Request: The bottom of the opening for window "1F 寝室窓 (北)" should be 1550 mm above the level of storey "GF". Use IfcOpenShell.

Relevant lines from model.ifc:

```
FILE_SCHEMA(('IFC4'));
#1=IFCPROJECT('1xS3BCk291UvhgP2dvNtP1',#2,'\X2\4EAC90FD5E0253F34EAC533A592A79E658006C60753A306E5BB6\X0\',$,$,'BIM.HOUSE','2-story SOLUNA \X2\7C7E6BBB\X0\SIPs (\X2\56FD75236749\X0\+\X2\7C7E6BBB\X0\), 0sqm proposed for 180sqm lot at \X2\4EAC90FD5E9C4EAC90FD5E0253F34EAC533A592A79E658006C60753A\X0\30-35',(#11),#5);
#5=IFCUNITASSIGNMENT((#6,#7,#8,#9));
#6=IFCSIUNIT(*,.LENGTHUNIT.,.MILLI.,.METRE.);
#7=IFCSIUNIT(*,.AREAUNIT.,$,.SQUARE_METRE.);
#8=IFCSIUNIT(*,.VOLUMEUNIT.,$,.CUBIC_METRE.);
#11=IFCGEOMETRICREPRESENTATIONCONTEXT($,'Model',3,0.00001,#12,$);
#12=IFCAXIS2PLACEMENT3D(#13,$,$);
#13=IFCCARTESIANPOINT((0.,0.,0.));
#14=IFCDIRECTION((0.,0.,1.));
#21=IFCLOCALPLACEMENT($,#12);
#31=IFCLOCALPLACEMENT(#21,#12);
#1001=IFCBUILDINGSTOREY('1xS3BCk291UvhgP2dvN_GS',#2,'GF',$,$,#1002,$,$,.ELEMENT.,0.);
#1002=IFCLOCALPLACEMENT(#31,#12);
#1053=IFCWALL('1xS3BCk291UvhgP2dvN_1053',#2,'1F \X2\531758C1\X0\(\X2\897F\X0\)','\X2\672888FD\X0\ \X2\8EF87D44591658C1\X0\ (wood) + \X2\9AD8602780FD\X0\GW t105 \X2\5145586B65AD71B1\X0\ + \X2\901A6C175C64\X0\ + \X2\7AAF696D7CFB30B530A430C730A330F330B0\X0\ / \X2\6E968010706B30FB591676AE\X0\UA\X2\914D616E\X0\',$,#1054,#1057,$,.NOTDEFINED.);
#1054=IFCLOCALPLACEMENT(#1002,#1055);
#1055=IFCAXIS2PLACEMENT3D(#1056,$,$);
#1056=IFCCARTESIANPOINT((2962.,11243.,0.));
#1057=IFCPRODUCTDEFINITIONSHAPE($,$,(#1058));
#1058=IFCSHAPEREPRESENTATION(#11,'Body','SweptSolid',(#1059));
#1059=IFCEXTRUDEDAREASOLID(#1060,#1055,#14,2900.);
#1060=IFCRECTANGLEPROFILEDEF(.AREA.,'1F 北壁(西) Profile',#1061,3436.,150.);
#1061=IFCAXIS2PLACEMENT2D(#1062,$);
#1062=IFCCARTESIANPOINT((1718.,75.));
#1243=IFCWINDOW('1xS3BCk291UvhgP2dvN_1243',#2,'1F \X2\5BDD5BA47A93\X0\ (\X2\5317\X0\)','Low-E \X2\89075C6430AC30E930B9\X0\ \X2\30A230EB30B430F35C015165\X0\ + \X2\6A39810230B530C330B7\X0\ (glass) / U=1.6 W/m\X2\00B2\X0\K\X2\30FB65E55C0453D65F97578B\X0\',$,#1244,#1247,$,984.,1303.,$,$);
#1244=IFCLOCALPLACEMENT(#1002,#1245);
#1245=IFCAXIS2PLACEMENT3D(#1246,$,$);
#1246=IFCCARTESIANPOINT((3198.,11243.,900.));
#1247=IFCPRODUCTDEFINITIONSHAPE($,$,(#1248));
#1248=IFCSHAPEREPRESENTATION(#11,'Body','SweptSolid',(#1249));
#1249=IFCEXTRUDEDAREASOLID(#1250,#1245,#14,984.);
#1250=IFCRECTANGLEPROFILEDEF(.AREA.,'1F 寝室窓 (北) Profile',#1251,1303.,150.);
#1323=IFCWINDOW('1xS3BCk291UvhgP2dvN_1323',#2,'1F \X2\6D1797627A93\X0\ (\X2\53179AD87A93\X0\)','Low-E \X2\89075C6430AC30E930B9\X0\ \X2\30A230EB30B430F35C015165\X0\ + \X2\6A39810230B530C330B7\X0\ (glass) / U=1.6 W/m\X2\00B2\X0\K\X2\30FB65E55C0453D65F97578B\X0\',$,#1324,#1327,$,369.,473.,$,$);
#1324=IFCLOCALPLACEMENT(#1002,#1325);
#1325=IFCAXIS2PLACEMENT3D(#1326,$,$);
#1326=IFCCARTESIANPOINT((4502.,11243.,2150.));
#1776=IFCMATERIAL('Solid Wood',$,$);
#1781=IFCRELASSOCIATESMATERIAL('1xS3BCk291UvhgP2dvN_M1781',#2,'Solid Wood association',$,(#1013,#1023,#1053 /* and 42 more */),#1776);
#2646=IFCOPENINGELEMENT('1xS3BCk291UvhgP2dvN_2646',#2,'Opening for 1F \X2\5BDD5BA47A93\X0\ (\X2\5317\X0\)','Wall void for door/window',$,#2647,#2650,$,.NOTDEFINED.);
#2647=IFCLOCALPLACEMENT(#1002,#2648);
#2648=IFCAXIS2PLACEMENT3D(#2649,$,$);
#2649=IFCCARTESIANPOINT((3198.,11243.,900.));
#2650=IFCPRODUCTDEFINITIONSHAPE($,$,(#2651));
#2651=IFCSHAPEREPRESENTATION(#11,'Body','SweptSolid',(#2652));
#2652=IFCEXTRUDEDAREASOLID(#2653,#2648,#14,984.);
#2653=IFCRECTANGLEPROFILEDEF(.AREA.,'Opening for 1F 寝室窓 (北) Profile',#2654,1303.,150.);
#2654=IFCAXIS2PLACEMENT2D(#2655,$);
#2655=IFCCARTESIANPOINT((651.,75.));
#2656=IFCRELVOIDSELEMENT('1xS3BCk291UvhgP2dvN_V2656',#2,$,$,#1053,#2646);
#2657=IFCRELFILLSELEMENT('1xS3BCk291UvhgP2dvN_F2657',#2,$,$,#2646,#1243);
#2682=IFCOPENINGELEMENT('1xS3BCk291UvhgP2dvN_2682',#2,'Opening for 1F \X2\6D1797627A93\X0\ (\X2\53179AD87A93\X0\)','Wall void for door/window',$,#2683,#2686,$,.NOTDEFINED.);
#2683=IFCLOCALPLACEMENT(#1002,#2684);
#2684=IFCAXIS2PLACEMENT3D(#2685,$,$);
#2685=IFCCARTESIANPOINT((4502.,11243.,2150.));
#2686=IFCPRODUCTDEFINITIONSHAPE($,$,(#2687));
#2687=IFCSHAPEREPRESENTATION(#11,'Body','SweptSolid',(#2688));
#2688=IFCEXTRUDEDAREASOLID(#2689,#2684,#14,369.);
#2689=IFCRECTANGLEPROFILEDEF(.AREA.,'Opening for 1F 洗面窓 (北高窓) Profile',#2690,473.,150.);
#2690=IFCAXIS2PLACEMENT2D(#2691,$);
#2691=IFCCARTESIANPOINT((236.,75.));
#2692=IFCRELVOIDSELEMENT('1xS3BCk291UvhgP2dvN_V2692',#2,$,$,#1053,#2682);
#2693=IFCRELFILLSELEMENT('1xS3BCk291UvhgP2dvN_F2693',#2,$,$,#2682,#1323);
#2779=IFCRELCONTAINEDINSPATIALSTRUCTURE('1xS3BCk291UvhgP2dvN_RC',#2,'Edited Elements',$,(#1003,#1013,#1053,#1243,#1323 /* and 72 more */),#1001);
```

```python
import numpy as np
import ifcopenshell
import ifcopenshell.api.geometry
import ifcopenshell.geom
import ifcopenshell.util.element
import ifcopenshell.util.placement
import ifcopenshell.util.shape
import ifcopenshell.util.unit

model = ifcopenshell.open("model.ifc")
unit_scale = ifcopenshell.util.unit.calculate_unit_scale(model)

window = model.by_guid("1xS3BCk291UvhgP2dvN_1243")
opening = window.FillsVoids[0].RelatingOpeningElement
storey = ifcopenshell.util.element.get_container(window, ifc_class="IfcBuildingStorey")
level = ifcopenshell.util.placement.get_local_placement(storey.ObjectPlacement)[2, 3]

# The opening's origin need not be at the sill, so measure its lowest point.
shape = ifcopenshell.geom.create_shape(ifcopenshell.geom.settings(), opening)
bottom = ifcopenshell.util.shape.get_shape_bottom_elevation(shape, shape.geometry) / unit_scale
dz = level + 1.55 / unit_scale - bottom

shift = np.array([0.0, 0.0, dz])
# The window is not placed relative to its opening, so move both.
for product in (opening, window):
    matrix = ifcopenshell.util.placement.get_local_placement(product.ObjectPlacement)
    matrix[:3, 3] += shift
    ifcopenshell.api.geometry.edit_object_placement(model, product=product, matrix=matrix, is_si=False)

print(f"moved by {dz * unit_scale:+.3f} m")

model.write("model_rev.ifc")
```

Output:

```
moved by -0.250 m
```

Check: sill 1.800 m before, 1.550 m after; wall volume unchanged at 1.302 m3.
